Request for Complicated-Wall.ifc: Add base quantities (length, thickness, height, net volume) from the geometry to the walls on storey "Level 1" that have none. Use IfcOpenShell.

First a look at what the model holds.

```python
import ifcopenshell
import ifcopenshell.util.element
import ifcopenshell.util.unit

model = ifcopenshell.open("Complicated-Wall.ifc")
print(model.schema)
for unit_type in ("LENGTHUNIT", "AREAUNIT", "VOLUMEUNIT"):
    print(unit_type, ifcopenshell.util.unit.calculate_unit_scale(model, unit_type))
storey = next(s for s in model.by_type("IfcBuildingStorey") if s.Name == "Level 1")
walls = [e for e in ifcopenshell.util.element.get_decomposition(storey) if e.is_a("IfcWall")]
for e in sorted(walls, key=lambda e: e.id()):
    print(e.id(), e.is_a(), e.Name, list(ifcopenshell.util.element.get_psets(e, qtos_only=True)), sep=" | ")
```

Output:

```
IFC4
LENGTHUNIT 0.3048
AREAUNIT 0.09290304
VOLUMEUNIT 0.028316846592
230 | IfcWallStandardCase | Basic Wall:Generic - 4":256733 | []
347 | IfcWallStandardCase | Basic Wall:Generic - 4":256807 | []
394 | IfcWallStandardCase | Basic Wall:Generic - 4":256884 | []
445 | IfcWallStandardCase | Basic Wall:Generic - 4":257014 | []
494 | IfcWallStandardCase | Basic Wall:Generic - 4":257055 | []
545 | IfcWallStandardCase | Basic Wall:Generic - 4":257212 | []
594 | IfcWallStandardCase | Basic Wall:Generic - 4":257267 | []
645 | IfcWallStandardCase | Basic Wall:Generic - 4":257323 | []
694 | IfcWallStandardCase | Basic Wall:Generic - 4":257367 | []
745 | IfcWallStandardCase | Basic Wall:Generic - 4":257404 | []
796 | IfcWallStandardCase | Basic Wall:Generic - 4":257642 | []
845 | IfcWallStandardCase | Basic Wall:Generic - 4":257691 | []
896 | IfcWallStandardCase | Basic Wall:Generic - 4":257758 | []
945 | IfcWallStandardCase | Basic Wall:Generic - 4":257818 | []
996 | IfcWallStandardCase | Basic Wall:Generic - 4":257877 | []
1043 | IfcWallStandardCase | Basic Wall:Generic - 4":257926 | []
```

```python
import ifcopenshell
import ifcopenshell.api.pset
import ifcopenshell.geom
import ifcopenshell.util.element
import ifcopenshell.util.shape
import ifcopenshell.util.unit

model = ifcopenshell.open("Complicated-Wall.ifc")
unit_scale = ifcopenshell.util.unit.calculate_unit_scale(model)
volume_scale = ifcopenshell.util.unit.calculate_unit_scale(model, "VOLUMEUNIT")
settings = ifcopenshell.geom.settings()

storey = next(s for s in model.by_type("IfcBuildingStorey") if s.Name == "Level 1")
walls = [e for e in ifcopenshell.util.element.get_decomposition(storey) if e.is_a("IfcWall")]

for e in sorted(walls, key=lambda e: e.id()):
    if ifcopenshell.util.element.get_psets(e, qtos_only=True, should_inherit=False):
        continue
    # Geometry comes back in metres, in the element's own axes.
    shape = ifcopenshell.geom.create_shape(settings, e)
    values = {
        "Length": ifcopenshell.util.shape.get_x(shape.geometry) / unit_scale,
        "Width": ifcopenshell.util.shape.get_y(shape.geometry) / unit_scale,
        "Height": ifcopenshell.util.shape.get_z(shape.geometry) / unit_scale,
        "NetVolume": ifcopenshell.util.shape.get_volume(shape.geometry) / volume_scale,
    }
    qto = ifcopenshell.api.pset.add_qto(model, product=e, name="Qto_WallBaseQuantities")
    ifcopenshell.api.pset.edit_qto(model, qto=qto, properties=values)
    print(e.id(), {k: round(v, 3) for k, v in values.items()})

model.write("Complicated-Wall-out.ifc")
```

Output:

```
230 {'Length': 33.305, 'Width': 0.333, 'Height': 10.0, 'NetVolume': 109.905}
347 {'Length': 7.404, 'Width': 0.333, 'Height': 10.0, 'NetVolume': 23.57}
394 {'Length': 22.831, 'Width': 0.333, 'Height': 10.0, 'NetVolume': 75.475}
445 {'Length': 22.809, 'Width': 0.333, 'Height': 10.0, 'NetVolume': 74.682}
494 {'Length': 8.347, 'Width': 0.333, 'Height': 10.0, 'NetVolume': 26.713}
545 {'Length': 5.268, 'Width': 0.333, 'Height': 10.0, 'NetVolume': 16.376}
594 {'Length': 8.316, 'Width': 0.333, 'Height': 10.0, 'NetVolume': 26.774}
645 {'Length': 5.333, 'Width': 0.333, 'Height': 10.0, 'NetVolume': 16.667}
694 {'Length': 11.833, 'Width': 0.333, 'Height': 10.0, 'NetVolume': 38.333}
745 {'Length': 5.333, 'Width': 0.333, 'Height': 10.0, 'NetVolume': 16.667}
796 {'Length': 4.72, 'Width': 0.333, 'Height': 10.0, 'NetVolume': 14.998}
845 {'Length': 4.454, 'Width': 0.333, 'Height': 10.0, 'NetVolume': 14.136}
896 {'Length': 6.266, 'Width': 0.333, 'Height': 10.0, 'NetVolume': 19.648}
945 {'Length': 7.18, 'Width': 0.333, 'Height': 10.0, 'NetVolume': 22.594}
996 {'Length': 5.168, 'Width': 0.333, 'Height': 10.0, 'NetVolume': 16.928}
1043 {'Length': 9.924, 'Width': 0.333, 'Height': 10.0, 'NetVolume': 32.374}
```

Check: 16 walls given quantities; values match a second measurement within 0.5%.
